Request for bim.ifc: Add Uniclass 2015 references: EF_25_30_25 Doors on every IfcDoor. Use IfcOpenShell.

First a look at what the model holds.

```python
import ifcopenshell

model = ifcopenshell.open("bim.ifc")
print(model.schema)
print("classifications:", [c.Name for c in model.by_type("IfcClassification")])
for ifc_class in ("IfcDoor", "IfcRoof", "IfcStair", "IfcWall", "IfcWindow"):
    print(ifc_class, len(model.by_type(ifc_class)))
```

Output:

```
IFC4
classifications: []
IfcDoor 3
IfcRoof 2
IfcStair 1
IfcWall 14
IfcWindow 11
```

```python
import ifcopenshell
import ifcopenshell.api.classification

model = ifcopenshell.open("bim.ifc")

system = ifcopenshell.api.classification.add_classification(model, classification="Uniclass 2015")

codes = {
    "IfcDoor": ("EF_25_30_25", "Doors"),
}
for ifc_class, (code, name) in codes.items():
    products = model.by_type(ifc_class)
    ifcopenshell.api.classification.add_reference(
        model, products=products, classification=system, identification=code, name=name
    )
    print(code, len(products))

model.write("bim_edited.ifc")
```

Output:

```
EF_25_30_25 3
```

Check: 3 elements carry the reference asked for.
